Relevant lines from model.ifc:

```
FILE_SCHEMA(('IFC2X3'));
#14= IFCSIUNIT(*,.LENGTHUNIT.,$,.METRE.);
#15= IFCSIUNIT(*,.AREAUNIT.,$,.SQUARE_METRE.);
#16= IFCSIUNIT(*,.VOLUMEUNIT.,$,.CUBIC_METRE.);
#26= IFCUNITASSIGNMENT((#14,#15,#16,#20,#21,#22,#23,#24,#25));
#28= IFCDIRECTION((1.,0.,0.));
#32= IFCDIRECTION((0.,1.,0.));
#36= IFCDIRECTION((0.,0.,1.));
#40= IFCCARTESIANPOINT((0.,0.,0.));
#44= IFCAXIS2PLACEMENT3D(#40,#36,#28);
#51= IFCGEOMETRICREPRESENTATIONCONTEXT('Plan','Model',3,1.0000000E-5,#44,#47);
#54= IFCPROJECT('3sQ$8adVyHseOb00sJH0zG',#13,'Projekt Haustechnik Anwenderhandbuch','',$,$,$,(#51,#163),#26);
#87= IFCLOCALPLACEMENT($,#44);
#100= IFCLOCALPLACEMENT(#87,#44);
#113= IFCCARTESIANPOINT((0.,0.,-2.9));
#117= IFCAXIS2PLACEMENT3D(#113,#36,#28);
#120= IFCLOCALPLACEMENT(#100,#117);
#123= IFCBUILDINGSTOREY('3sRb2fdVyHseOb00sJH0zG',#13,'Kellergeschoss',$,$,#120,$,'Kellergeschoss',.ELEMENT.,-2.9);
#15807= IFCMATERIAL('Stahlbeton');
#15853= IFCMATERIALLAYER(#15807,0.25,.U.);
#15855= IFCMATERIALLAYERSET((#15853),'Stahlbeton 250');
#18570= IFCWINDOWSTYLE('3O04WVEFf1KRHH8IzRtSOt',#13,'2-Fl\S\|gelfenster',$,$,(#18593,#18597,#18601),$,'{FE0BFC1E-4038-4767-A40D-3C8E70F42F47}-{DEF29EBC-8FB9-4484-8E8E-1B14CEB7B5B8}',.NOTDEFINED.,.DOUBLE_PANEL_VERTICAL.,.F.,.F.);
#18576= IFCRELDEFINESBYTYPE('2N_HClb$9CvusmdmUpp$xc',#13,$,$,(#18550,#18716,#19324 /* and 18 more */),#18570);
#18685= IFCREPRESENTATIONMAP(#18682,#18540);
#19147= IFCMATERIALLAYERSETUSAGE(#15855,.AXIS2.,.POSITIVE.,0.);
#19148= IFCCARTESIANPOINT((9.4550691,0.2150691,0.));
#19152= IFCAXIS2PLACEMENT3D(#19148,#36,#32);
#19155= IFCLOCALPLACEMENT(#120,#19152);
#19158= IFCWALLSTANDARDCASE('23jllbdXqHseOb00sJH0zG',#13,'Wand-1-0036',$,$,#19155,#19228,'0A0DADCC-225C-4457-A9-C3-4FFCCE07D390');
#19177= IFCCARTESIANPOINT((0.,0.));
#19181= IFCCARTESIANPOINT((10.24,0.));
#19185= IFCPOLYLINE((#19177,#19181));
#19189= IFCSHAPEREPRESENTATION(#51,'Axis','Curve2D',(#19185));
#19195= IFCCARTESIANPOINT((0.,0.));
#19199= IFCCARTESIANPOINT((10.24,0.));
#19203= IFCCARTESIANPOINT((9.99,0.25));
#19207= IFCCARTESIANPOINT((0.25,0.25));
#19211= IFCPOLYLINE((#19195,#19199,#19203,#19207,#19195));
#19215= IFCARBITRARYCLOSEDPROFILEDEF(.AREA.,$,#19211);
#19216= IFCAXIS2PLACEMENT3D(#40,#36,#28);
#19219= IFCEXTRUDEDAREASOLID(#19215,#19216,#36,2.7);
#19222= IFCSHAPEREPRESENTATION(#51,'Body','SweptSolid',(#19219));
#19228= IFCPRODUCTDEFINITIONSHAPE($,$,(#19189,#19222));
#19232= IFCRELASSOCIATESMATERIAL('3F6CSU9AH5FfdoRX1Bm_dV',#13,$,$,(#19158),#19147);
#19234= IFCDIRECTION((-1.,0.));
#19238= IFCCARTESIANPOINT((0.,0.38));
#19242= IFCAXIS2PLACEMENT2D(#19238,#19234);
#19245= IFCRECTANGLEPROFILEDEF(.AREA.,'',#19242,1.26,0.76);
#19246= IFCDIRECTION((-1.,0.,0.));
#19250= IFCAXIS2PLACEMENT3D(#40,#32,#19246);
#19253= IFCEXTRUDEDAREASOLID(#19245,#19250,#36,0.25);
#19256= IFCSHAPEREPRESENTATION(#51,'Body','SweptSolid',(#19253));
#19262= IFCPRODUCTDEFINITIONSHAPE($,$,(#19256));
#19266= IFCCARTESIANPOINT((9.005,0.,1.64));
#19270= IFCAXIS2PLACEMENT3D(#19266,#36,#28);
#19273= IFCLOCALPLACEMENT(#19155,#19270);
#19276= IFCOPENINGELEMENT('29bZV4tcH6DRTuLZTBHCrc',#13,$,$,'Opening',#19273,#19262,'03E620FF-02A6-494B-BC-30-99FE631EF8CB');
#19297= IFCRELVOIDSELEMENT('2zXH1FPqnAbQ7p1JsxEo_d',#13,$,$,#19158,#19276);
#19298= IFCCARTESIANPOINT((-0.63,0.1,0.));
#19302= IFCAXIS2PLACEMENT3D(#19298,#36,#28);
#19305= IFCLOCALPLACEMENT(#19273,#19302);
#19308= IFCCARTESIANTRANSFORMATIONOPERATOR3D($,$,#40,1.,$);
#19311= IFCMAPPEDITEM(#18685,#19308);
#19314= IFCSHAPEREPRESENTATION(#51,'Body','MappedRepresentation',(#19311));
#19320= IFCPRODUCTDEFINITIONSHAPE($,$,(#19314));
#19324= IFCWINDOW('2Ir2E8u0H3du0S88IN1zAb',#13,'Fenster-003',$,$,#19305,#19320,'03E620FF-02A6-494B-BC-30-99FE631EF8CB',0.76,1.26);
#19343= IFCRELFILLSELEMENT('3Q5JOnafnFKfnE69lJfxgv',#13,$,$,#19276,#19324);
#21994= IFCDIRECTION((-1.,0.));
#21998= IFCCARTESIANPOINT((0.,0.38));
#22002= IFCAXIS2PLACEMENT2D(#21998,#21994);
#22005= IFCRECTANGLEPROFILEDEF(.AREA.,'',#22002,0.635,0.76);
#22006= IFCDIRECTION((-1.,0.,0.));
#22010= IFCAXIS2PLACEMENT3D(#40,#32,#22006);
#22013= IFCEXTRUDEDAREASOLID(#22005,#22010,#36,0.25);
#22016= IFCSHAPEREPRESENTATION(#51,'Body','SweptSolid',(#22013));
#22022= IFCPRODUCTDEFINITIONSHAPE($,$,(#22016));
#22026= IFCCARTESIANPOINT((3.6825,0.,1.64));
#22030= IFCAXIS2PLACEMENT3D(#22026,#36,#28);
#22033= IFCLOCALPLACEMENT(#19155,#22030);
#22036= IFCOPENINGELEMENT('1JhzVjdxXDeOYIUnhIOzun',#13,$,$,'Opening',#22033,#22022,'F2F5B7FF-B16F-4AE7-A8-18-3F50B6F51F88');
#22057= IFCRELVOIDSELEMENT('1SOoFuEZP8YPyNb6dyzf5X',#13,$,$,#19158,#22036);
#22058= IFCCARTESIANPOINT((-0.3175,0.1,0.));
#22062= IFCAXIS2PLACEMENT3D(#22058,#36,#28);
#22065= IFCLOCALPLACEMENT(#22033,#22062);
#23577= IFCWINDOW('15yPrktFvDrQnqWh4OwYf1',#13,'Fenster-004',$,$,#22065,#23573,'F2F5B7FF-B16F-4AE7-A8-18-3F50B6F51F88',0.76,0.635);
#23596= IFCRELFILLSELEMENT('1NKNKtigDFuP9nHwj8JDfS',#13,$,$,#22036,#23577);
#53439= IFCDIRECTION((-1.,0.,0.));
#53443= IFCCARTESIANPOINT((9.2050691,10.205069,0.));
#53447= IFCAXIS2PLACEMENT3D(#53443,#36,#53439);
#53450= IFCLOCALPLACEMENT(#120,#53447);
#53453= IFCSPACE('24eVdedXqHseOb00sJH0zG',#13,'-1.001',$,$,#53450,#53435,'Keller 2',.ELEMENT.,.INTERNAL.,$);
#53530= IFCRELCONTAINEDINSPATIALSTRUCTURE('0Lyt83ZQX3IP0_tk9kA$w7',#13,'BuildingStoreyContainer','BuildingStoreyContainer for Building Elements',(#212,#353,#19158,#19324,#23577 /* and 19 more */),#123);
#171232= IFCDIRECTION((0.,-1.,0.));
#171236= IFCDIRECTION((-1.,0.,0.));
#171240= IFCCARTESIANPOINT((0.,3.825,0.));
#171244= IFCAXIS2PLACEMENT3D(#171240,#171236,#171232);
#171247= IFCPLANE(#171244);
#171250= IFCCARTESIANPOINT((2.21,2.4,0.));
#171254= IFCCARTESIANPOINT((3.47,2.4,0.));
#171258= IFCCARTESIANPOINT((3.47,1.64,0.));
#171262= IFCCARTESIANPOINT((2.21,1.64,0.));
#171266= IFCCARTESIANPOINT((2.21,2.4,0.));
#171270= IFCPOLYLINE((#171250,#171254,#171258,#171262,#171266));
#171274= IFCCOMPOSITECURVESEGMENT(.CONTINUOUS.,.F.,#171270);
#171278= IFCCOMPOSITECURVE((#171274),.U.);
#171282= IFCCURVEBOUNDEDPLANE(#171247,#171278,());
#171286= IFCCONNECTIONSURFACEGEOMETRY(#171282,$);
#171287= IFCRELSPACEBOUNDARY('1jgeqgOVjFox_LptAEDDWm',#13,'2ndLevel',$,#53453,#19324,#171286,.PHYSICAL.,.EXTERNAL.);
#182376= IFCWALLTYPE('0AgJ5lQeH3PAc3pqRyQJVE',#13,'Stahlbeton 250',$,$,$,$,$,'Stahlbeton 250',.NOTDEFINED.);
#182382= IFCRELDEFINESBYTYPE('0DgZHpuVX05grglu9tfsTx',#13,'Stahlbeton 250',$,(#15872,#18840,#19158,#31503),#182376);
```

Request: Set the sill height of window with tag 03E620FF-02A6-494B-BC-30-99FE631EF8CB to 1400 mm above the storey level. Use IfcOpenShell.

```python
import numpy as np
import ifcopenshell
import ifcopenshell.api.geometry
import ifcopenshell.geom
import ifcopenshell.util.element
import ifcopenshell.util.placement
import ifcopenshell.util.shape
import ifcopenshell.util.unit

model = ifcopenshell.open("model.ifc")
unit_scale = ifcopenshell.util.unit.calculate_unit_scale(model)

window = model.by_id(19324)
opening = window.FillsVoids[0].RelatingOpeningElement
storey = ifcopenshell.util.element.get_container(window, ifc_class="IfcBuildingStorey")
level = ifcopenshell.util.placement.get_local_placement(storey.ObjectPlacement)[2, 3]

# The opening's origin need not be at the sill, so measure its lowest point.
shape = ifcopenshell.geom.create_shape(ifcopenshell.geom.settings(), opening)
bottom = ifcopenshell.util.shape.get_shape_bottom_elevation(shape, shape.geometry) / unit_scale
dz = level + 1.4 / unit_scale - bottom

shift = np.array([0.0, 0.0, dz])
# The window is placed relative to its opening, so it follows when the opening moves.
matrix = ifcopenshell.util.placement.get_local_placement(opening.ObjectPlacement)
matrix[:3, 3] += shift
ifcopenshell.api.geometry.edit_object_placement(
    model, product=opening, matrix=matrix, is_si=False, should_transform_children=True
)

# Space boundary surfaces are stored in each space's coordinates; move them too.
for rel in window.ProvidesBoundaries:
    if not rel.ConnectionGeometry:
        continue
    surface = rel.ConnectionGeometry.SurfaceOnRelatingElement.BasisSurface
    space_matrix = ifcopenshell.util.placement.get_local_placement(rel.RelatingSpace.ObjectPlacement)
    point = np.array(surface.Position.Location.Coordinates) + space_matrix[:3, :3].T @ shift
    surface.Position = model.createIfcAxis2Placement3D(
        model.createIfcCartesianPoint(point.tolist()), surface.Position.Axis, surface.Position.RefDirection
    )

print(f"moved by {dz * unit_scale:+.3f} m")

model.write("model_edited.ifc")
```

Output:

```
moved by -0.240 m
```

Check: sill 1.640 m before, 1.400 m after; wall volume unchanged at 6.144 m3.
